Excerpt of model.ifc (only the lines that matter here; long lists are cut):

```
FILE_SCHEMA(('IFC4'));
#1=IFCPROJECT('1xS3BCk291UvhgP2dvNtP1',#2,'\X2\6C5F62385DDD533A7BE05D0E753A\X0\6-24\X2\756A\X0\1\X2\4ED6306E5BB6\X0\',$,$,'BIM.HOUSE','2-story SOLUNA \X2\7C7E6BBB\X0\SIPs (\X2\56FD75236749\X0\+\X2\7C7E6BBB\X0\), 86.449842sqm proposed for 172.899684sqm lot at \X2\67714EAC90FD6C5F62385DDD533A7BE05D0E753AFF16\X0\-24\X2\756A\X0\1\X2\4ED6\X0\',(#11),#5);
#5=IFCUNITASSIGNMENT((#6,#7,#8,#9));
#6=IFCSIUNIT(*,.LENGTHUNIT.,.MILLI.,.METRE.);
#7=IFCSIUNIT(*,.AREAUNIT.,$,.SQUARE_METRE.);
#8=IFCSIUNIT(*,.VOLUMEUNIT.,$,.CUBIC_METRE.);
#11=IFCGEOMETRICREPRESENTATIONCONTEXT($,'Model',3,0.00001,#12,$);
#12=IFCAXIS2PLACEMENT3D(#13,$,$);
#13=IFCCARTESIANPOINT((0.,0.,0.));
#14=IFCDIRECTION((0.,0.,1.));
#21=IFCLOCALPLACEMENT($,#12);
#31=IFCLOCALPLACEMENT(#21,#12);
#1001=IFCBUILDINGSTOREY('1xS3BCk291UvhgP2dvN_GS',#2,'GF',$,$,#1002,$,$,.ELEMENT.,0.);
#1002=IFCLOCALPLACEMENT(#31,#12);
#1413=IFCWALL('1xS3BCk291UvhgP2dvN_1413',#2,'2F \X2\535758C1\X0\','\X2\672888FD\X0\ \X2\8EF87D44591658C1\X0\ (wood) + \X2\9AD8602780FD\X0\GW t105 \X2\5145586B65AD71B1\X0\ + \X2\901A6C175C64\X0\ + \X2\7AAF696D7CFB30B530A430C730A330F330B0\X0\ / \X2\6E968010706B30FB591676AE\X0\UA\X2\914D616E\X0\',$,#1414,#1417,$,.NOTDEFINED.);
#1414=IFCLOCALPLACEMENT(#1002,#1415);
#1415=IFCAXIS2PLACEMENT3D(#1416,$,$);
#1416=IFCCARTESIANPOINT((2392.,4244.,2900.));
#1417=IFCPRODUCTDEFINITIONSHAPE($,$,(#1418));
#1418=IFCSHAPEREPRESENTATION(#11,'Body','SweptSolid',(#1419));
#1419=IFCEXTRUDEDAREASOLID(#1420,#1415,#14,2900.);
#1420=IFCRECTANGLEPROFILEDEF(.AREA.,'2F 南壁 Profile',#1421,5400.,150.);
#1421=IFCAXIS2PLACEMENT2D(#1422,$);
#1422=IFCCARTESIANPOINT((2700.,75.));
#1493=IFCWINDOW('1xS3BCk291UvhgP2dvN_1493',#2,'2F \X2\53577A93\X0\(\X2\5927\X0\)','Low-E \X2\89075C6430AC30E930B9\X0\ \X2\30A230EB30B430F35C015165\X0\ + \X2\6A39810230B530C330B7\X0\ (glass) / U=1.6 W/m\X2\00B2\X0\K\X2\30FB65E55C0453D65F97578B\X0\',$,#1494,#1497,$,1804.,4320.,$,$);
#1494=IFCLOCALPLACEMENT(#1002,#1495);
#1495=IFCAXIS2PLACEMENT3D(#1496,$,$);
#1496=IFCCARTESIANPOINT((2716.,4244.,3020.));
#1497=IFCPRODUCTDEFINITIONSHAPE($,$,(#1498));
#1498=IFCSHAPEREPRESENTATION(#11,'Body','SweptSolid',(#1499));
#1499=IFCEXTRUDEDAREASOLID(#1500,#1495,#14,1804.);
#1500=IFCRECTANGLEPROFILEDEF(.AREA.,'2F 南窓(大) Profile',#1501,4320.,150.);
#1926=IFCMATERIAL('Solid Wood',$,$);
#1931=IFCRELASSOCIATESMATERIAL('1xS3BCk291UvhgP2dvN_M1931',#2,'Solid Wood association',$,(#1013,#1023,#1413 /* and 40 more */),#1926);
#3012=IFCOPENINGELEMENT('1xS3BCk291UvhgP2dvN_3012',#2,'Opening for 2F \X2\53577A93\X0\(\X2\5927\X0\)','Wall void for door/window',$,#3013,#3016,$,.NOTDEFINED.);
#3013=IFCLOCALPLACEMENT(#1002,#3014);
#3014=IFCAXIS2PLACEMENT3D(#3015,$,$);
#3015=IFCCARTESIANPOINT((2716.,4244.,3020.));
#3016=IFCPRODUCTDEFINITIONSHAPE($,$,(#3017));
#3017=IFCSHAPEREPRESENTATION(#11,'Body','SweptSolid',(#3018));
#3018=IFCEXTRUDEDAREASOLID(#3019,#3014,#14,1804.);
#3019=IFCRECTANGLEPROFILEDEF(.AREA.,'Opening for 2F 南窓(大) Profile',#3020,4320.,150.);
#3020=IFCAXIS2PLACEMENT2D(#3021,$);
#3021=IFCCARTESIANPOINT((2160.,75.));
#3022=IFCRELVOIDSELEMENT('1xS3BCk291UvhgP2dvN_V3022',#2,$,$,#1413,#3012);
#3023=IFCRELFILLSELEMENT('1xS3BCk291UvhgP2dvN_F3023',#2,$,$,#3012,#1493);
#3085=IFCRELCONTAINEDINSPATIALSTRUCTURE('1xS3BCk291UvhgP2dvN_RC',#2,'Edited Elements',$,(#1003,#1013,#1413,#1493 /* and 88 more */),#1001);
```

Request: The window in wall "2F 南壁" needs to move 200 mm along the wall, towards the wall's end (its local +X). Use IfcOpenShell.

```python
import ifcopenshell
import ifcopenshell.api.geometry
import ifcopenshell.util.placement

model = ifcopenshell.open("model.ifc")

window = model.by_guid("1xS3BCk291UvhgP2dvN_1493")
opening = window.FillsVoids[0].RelatingOpeningElement
wall = opening.VoidsElements[0].RelatingBuildingElement

wall_matrix = ifcopenshell.util.placement.get_local_placement(wall.ObjectPlacement)
shift = wall_matrix[:3, 0] * 200.0
before = ifcopenshell.util.placement.get_local_placement(window.ObjectPlacement)[:3, 3].copy()

# The window is not placed relative to its opening, so move both.
for product in (opening, window):
    matrix = ifcopenshell.util.placement.get_local_placement(product.ObjectPlacement)
    matrix[:3, 3] += shift
    ifcopenshell.api.geometry.edit_object_placement(model, product=product, matrix=matrix, is_si=False)

after = ifcopenshell.util.placement.get_local_placement(window.ObjectPlacement)[:3, 3]
print("window moved by", (after - before).round(3) + 0.0)

model.write("model_rev.ifc")
```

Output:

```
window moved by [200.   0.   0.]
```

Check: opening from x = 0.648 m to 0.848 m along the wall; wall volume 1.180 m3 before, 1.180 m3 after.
